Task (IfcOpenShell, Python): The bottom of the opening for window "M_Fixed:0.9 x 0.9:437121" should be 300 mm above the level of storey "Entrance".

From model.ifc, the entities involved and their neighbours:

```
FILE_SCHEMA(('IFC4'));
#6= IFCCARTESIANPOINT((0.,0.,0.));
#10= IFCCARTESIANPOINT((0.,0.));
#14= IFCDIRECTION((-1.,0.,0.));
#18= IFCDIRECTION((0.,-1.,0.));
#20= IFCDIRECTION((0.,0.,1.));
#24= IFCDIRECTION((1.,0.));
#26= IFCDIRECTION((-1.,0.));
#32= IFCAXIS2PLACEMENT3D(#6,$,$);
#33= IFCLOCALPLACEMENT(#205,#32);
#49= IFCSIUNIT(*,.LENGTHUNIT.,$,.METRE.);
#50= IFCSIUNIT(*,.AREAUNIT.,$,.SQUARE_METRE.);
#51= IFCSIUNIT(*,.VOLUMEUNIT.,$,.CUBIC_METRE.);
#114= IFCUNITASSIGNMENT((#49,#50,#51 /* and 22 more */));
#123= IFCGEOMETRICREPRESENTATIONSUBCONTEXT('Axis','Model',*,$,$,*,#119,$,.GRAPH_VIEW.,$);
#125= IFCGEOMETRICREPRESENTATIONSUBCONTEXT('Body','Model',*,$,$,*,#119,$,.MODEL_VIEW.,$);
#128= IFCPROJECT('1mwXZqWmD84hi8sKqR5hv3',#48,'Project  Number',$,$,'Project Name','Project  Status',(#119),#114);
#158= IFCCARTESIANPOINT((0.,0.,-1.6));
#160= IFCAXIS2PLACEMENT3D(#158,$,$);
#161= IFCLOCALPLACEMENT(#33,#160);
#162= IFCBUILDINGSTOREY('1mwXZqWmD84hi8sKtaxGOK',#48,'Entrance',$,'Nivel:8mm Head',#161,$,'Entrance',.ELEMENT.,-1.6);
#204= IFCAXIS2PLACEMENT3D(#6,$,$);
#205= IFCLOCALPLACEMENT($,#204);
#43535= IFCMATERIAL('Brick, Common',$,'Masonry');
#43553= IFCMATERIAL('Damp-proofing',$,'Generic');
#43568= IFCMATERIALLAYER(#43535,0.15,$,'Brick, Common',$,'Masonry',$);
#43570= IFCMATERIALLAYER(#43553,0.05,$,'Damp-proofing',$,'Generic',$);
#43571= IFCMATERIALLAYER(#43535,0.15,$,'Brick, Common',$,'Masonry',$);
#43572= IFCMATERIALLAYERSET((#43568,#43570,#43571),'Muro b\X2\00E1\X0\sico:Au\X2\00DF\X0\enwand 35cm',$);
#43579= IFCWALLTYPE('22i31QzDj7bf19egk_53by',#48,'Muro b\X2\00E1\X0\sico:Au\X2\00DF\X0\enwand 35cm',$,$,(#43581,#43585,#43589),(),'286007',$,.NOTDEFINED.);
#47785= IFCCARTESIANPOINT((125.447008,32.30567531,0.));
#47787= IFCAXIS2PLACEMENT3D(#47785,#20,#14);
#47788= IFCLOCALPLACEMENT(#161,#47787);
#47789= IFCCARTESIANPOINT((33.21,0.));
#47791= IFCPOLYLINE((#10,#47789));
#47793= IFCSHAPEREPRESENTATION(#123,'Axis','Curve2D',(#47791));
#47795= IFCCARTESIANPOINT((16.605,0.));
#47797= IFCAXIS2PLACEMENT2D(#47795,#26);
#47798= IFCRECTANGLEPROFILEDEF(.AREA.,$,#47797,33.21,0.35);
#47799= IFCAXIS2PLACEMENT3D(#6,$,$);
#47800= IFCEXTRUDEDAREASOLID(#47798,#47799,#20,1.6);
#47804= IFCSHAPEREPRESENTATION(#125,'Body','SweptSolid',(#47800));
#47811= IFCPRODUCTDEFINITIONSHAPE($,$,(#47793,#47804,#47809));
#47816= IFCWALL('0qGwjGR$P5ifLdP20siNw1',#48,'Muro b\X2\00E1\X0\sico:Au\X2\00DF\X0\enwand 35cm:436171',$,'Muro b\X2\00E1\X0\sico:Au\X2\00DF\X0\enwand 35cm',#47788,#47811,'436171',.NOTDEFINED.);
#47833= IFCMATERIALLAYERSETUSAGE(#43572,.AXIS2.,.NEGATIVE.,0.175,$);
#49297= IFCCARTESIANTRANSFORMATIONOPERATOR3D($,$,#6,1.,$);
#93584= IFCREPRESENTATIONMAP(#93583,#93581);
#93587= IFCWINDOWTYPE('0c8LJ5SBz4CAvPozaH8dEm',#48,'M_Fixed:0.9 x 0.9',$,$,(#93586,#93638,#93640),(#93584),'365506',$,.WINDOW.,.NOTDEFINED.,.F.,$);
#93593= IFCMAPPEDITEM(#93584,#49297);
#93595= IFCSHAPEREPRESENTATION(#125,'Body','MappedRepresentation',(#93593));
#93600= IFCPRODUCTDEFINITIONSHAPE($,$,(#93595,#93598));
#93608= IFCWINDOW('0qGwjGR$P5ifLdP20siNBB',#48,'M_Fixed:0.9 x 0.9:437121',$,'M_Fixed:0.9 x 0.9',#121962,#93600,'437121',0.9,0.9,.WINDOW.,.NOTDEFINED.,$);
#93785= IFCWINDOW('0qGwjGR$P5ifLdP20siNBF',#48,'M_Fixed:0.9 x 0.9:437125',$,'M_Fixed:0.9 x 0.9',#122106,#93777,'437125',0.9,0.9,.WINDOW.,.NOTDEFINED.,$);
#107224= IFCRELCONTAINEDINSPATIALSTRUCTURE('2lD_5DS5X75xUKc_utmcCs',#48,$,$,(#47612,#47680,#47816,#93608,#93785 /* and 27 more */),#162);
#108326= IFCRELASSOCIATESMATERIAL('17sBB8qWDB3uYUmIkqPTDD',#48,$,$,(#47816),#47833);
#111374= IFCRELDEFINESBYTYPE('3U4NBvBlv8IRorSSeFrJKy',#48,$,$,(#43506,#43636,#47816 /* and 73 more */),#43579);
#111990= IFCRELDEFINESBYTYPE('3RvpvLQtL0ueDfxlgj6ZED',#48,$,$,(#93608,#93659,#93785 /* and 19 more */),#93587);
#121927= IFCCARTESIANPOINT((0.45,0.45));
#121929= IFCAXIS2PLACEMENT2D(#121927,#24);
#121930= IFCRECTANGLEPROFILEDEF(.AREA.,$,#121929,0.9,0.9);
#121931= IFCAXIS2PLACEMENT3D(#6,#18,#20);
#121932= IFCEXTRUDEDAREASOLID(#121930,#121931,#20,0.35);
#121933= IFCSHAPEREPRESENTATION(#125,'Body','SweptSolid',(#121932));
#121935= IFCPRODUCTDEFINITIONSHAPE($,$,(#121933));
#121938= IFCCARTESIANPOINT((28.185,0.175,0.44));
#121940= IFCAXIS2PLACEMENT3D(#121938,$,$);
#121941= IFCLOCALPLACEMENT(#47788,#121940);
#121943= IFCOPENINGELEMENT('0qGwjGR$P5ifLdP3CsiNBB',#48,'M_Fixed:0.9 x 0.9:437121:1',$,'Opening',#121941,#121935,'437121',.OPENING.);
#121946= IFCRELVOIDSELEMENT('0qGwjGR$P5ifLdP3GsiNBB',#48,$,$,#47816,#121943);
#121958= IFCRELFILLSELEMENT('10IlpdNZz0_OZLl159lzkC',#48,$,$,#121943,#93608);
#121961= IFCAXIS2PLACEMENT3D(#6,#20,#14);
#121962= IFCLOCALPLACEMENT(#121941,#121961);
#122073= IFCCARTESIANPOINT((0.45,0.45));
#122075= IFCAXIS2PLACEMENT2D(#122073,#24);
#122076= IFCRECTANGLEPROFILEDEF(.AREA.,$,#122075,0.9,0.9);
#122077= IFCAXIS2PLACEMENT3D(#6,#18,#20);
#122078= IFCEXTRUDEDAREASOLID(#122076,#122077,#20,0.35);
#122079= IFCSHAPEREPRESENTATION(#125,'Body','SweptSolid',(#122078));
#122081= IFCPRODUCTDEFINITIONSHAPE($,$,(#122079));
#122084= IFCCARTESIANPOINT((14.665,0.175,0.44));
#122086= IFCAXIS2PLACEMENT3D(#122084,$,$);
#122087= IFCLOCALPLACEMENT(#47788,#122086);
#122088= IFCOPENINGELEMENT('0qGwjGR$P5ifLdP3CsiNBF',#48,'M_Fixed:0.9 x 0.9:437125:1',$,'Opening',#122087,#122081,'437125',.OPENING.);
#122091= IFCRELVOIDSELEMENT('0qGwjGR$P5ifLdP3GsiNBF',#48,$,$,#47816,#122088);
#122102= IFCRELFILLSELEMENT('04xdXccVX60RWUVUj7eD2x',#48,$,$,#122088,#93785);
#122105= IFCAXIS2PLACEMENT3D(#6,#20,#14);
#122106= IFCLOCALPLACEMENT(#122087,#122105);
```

```python
import numpy as np
import ifcopenshell
import ifcopenshell.api.geometry
import ifcopenshell.geom
import ifcopenshell.util.element
import ifcopenshell.util.placement
import ifcopenshell.util.shape
import ifcopenshell.util.unit

model = ifcopenshell.open("model.ifc")
unit_scale = ifcopenshell.util.unit.calculate_unit_scale(model)

window = model.by_guid("0qGwjGR$P5ifLdP20siNBB")
opening = window.FillsVoids[0].RelatingOpeningElement
storey = ifcopenshell.util.element.get_container(window, ifc_class="IfcBuildingStorey")
level = ifcopenshell.util.placement.get_local_placement(storey.ObjectPlacement)[2, 3]

# The opening's origin need not be at the sill, so measure its lowest point.
shape = ifcopenshell.geom.create_shape(ifcopenshell.geom.settings(), opening)
bottom = ifcopenshell.util.shape.get_shape_bottom_elevation(shape, shape.geometry) / unit_scale
dz = level + 0.3 - bottom

shift = np.array([0.0, 0.0, dz])
# The window is placed relative to its opening, so it follows when the opening moves.
matrix = ifcopenshell.util.placement.get_local_placement(opening.ObjectPlacement)
matrix[:3, 3] += shift
ifcopenshell.api.geometry.edit_object_placement(
    model, product=opening, matrix=matrix, is_si=False, should_transform_children=True
)

print(f"moved by {dz * unit_scale:+.3f} m")

model.write("model_v2.ifc")
```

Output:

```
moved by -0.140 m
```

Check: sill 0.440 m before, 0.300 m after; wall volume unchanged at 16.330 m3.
